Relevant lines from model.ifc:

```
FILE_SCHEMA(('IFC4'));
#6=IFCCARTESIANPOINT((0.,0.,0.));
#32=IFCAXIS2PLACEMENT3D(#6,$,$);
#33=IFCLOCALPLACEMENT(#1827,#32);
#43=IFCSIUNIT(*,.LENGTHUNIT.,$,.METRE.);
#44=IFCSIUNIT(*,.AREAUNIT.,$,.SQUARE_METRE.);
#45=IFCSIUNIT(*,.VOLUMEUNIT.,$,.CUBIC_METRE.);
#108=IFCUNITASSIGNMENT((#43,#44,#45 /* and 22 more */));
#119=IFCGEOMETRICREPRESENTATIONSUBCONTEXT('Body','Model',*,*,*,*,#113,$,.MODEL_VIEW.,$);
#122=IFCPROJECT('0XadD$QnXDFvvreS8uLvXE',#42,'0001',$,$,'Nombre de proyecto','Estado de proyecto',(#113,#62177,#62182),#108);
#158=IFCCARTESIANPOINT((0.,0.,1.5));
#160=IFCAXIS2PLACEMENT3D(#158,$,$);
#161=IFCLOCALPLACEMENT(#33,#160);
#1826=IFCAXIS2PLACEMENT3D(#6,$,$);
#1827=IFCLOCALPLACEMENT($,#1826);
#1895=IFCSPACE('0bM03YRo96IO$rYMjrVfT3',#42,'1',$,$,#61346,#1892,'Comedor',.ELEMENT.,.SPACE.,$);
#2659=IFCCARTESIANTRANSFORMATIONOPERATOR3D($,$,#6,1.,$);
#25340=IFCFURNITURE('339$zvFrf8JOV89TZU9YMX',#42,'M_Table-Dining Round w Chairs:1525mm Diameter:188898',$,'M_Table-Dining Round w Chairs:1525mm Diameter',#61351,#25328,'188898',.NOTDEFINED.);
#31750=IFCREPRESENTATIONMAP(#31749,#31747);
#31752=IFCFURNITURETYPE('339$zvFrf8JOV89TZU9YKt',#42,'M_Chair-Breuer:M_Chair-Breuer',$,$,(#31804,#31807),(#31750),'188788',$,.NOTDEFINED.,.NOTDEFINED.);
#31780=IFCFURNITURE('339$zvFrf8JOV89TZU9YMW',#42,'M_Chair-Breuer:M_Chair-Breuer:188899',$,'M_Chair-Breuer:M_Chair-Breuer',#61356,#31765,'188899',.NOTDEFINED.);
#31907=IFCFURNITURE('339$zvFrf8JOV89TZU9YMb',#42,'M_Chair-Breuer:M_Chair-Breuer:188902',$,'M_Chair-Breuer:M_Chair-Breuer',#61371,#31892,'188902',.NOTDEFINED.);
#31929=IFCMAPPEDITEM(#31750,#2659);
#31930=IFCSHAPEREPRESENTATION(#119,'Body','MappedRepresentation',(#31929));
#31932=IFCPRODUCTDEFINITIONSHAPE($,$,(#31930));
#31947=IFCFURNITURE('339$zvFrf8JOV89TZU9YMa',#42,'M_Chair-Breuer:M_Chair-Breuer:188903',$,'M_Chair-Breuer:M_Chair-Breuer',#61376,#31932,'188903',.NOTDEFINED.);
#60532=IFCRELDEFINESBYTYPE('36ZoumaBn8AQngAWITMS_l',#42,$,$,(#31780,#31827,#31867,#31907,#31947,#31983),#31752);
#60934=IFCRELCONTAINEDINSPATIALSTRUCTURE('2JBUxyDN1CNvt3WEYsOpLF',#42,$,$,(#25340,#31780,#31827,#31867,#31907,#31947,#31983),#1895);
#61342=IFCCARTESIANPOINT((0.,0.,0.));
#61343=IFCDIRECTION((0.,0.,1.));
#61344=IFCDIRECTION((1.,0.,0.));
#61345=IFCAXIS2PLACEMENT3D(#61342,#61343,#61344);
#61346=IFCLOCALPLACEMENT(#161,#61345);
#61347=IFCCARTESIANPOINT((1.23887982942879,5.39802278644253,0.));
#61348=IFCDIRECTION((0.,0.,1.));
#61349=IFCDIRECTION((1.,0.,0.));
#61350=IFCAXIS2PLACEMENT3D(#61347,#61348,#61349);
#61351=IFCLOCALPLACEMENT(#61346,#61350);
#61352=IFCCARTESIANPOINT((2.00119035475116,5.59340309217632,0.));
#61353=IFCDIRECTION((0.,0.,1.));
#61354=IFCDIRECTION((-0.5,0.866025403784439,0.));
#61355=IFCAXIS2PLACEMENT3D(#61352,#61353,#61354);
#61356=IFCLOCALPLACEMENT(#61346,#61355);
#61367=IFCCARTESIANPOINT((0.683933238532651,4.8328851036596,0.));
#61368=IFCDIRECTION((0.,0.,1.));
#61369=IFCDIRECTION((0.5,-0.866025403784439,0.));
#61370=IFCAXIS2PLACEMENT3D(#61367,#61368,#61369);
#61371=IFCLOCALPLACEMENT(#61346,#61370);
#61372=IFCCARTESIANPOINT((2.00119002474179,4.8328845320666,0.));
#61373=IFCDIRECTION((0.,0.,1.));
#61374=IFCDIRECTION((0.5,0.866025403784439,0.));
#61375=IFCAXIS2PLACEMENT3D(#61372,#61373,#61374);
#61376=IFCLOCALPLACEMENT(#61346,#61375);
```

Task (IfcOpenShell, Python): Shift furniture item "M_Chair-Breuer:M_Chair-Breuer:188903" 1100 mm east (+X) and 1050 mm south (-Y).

```python
import ifcopenshell
import ifcopenshell.api.geometry
import ifcopenshell.util.placement
import ifcopenshell.util.unit

model = ifcopenshell.open("model.ifc")
unit_scale = ifcopenshell.util.unit.calculate_unit_scale(model)

item = model.by_guid("339$zvFrf8JOV89TZU9YMa")
matrix = ifcopenshell.util.placement.get_local_placement(item.ObjectPlacement)
matrix[0, 3] += 1.1 / unit_scale
matrix[1, 3] -= 1.05 / unit_scale
ifcopenshell.api.geometry.edit_object_placement(model, product=item, matrix=matrix, is_si=False)

print(ifcopenshell.util.placement.get_local_placement(item.ObjectPlacement).round(3) + 0.0)

model.write("model_v2.ifc")
```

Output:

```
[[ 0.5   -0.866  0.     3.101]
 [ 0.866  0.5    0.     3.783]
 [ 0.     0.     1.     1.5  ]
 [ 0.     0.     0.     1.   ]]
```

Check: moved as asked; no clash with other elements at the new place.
